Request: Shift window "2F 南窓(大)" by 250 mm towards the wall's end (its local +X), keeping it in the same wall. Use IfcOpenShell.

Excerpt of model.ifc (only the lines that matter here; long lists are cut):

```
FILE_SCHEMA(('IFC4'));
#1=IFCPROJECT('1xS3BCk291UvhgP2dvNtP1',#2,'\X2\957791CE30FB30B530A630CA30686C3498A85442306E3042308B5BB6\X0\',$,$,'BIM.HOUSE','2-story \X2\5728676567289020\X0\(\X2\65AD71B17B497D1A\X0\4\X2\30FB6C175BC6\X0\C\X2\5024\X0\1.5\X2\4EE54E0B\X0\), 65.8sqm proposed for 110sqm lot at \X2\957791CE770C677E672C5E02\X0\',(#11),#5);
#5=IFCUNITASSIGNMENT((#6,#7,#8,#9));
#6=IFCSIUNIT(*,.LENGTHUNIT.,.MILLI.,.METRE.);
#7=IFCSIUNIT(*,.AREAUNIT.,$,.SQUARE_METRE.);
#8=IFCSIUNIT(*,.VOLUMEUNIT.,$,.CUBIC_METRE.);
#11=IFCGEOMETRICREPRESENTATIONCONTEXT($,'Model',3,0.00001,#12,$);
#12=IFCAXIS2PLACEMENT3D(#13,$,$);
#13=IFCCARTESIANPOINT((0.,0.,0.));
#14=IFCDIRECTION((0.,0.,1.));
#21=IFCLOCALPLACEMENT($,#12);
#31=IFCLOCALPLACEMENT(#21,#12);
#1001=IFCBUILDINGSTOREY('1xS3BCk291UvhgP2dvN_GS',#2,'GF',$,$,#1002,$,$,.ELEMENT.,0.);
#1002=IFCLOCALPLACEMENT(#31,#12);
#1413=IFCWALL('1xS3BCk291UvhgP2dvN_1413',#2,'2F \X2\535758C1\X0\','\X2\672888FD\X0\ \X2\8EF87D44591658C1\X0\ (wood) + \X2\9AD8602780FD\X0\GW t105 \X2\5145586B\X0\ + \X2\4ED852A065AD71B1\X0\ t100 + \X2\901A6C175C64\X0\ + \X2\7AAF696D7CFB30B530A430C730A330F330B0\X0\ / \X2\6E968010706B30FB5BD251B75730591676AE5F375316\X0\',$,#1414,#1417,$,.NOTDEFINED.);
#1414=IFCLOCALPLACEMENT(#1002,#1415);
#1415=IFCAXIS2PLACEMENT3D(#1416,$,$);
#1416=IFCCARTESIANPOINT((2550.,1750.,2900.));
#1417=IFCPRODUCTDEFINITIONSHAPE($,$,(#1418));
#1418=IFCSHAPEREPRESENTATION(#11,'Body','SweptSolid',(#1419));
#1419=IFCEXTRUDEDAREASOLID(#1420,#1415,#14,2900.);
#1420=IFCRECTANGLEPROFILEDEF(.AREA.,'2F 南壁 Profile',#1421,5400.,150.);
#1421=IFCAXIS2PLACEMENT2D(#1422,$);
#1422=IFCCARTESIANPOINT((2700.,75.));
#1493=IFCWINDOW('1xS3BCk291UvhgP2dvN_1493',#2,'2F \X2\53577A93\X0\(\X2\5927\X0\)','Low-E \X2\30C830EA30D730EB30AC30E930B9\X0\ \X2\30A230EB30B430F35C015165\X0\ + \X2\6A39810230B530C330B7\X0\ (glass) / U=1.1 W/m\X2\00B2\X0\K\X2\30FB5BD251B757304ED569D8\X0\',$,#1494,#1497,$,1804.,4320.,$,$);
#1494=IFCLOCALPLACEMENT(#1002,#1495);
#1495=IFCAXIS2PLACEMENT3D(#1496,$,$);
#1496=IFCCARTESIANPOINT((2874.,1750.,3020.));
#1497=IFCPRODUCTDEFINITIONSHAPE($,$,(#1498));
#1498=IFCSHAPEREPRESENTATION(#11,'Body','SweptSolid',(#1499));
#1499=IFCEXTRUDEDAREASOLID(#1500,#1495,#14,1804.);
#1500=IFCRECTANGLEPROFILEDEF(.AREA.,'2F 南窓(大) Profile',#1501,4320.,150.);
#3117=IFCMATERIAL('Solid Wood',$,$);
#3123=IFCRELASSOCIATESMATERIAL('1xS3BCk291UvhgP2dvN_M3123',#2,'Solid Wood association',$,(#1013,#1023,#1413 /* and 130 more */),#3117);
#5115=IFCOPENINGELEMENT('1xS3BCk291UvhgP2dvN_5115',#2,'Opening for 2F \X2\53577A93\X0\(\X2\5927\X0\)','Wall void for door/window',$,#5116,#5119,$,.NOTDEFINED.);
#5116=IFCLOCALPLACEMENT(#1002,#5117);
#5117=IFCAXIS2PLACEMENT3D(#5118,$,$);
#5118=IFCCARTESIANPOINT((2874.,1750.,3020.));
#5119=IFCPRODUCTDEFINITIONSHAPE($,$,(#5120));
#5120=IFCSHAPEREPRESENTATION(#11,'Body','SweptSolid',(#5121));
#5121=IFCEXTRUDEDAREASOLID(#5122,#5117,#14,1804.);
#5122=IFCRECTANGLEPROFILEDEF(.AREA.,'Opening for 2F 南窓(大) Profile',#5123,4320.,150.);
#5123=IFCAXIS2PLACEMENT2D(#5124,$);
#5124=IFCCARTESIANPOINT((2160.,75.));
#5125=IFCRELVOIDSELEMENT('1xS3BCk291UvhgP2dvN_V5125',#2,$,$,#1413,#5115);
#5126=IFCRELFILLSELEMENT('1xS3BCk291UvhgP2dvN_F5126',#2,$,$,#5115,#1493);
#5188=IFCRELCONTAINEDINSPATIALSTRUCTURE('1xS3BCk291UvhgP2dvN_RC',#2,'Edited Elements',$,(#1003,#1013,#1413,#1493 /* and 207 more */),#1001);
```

```python
import ifcopenshell
import ifcopenshell.api.geometry
import ifcopenshell.util.placement

model = ifcopenshell.open("model.ifc")

window = model.by_guid("1xS3BCk291UvhgP2dvN_1493")
opening = window.FillsVoids[0].RelatingOpeningElement
wall = opening.VoidsElements[0].RelatingBuildingElement

wall_matrix = ifcopenshell.util.placement.get_local_placement(wall.ObjectPlacement)
shift = wall_matrix[:3, 0] * 250.0
before = ifcopenshell.util.placement.get_local_placement(window.ObjectPlacement)[:3, 3].copy()

# The window is not placed relative to its opening, so move both.
for product in (opening, window):
    matrix = ifcopenshell.util.placement.get_local_placement(product.ObjectPlacement)
    matrix[:3, 3] += shift
    ifcopenshell.api.geometry.edit_object_placement(model, product=product, matrix=matrix, is_si=False)

after = ifcopenshell.util.placement.get_local_placement(window.ObjectPlacement)[:3, 3]
print("window moved by", (after - before).round(3) + 0.0)

model.write("model_edited.ifc")
```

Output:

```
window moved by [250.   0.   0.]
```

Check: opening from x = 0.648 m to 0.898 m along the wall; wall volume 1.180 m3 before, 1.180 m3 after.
